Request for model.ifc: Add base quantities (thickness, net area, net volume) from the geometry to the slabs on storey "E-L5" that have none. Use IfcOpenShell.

First a look at what the model holds.

```python
import ifcopenshell
import ifcopenshell.util.element
import ifcopenshell.util.unit

model = ifcopenshell.open("model.ifc")
print(model.schema)
for unit_type in ("LENGTHUNIT", "AREAUNIT", "VOLUMEUNIT"):
    print(unit_type, ifcopenshell.util.unit.calculate_unit_scale(model, unit_type))
storey = next(s for s in model.by_type("IfcBuildingStorey") if s.Name == "E-L5")
slabs = [e for e in ifcopenshell.util.element.get_decomposition(storey) if e.is_a("IfcSlab")]
for e in sorted(slabs, key=lambda e: e.id()):
    print(e.id(), e.is_a(), e.Name, list(ifcopenshell.util.element.get_psets(e, qtos_only=True)), sep=" | ")
```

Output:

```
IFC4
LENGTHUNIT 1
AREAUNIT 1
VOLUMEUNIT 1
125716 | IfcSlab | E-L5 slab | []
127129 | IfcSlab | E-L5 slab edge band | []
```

```python
import ifcopenshell
import ifcopenshell.api.pset
import ifcopenshell.geom
import ifcopenshell.util.element
import ifcopenshell.util.shape
import ifcopenshell.util.unit

model = ifcopenshell.open("model.ifc")
unit_scale = ifcopenshell.util.unit.calculate_unit_scale(model)
area_scale = ifcopenshell.util.unit.calculate_unit_scale(model, "AREAUNIT")
volume_scale = ifcopenshell.util.unit.calculate_unit_scale(model, "VOLUMEUNIT")
settings = ifcopenshell.geom.settings()

storey = next(s for s in model.by_type("IfcBuildingStorey") if s.Name == "E-L5")
slabs = [e for e in ifcopenshell.util.element.get_decomposition(storey) if e.is_a("IfcSlab")]

for e in sorted(slabs, key=lambda e: e.id()):
    if ifcopenshell.util.element.get_psets(e, qtos_only=True, should_inherit=False):
        continue
    # Geometry comes back in metres, in the element's own axes.
    shape = ifcopenshell.geom.create_shape(settings, e)
    values = {
        "Width": ifcopenshell.util.shape.get_z(shape.geometry) / unit_scale,
        "NetArea": ifcopenshell.util.shape.get_footprint_area(shape.geometry) / area_scale,
        "NetVolume": ifcopenshell.util.shape.get_volume(shape.geometry) / volume_scale,
    }
    qto = ifcopenshell.api.pset.add_qto(model, product=e, name="Qto_SlabBaseQuantities")
    ifcopenshell.api.pset.edit_qto(model, qto=qto, properties=values)
    print(e.id(), {k: round(v, 3) for k, v in values.items()})

model.write("model-out.ifc")
```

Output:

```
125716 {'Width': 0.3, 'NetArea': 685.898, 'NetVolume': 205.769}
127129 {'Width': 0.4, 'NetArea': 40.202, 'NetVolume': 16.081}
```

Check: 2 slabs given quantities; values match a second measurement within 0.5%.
